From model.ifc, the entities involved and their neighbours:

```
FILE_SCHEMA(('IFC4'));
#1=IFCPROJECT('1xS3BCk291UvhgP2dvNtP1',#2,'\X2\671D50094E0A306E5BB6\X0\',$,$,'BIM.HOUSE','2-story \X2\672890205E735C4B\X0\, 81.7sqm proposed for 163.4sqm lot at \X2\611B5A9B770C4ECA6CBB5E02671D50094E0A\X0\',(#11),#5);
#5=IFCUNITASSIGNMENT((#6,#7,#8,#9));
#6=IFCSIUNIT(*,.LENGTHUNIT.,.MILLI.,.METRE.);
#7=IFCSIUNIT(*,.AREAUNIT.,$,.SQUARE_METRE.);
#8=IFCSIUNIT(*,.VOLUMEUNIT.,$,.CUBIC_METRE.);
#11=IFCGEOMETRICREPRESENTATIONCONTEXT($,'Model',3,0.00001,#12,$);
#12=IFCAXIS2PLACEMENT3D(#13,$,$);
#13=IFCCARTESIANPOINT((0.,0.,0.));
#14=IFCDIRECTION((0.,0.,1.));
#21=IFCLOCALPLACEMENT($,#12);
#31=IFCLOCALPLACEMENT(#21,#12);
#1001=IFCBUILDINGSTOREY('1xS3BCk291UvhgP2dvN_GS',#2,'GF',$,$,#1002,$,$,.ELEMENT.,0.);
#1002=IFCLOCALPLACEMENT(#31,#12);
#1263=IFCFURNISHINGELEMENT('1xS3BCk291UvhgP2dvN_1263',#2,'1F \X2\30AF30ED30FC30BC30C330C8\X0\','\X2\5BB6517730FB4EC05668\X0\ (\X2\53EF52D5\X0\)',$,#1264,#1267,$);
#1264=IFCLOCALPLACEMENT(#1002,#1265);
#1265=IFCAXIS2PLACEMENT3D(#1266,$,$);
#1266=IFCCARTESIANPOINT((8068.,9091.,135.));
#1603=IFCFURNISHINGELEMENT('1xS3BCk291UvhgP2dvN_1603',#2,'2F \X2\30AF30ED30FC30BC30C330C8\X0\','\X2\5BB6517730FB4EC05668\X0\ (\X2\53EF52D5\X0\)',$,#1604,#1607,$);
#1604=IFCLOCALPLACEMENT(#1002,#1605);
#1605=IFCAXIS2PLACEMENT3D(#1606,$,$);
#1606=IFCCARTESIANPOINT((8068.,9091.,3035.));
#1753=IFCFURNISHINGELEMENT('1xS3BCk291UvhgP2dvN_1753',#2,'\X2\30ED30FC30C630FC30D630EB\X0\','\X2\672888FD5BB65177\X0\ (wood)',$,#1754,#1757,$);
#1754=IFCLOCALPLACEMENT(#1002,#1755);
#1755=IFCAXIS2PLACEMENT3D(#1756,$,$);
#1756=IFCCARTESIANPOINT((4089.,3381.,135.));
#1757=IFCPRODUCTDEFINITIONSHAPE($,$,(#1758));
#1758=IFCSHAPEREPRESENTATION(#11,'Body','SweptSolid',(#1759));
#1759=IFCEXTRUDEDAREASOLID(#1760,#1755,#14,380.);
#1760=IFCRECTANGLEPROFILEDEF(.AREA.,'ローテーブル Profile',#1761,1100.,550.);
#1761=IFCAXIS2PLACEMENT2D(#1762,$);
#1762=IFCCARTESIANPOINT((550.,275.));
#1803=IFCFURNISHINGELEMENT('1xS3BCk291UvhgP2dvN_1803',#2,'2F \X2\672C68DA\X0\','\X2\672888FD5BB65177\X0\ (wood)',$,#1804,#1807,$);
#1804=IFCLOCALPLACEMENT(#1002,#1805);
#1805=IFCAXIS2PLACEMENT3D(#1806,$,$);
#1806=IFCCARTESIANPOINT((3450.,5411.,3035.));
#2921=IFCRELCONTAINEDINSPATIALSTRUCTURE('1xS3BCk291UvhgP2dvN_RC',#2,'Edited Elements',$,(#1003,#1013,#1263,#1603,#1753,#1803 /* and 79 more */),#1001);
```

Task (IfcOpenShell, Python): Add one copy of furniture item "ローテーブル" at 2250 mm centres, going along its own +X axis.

```python
import ifcopenshell
import ifcopenshell.api.geometry
import ifcopenshell.api.root
import ifcopenshell.util.element
import ifcopenshell.util.placement
import ifcopenshell.util.unit

model = ifcopenshell.open("model.ifc")
unit_scale = ifcopenshell.util.unit.calculate_unit_scale(model)


def reuse_history(source, copy):
    """copy_class also copies each property set's owner history, people and application; keep the originals."""
    for rel in copy.IsDefinedBy:
        if rel.is_a("IfcRelDefinesByProperties") and (history := rel.RelatingPropertyDefinition.OwnerHistory):
            rel.RelatingPropertyDefinition.OwnerHistory = source.OwnerHistory
            ifcopenshell.util.element.remove_deep2(model, history)


source = model.by_guid("1xS3BCk291UvhgP2dvN_1753")
base = ifcopenshell.util.placement.get_local_placement(source.ObjectPlacement)
step = base[:3, 0] * 2.25 / unit_scale

for i in range(1, 2):
    copy = ifcopenshell.api.root.copy_class(model, product=source)
    copy.Representation = ifcopenshell.util.element.copy_deep(
        model, source.Representation, exclude=["IfcGeometricRepresentationContext", "IfcRepresentationMap"]
    )
    reuse_history(source, copy)
    matrix = base.copy()
    matrix[:3, 3] += i * step
    print("added at", matrix[:3, 3].round(3) + 0.0)
    ifcopenshell.api.geometry.edit_object_placement(model, product=copy, matrix=matrix, is_si=False)

model.write("model_updated.ifc")
```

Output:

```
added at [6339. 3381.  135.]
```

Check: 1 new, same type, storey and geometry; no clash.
